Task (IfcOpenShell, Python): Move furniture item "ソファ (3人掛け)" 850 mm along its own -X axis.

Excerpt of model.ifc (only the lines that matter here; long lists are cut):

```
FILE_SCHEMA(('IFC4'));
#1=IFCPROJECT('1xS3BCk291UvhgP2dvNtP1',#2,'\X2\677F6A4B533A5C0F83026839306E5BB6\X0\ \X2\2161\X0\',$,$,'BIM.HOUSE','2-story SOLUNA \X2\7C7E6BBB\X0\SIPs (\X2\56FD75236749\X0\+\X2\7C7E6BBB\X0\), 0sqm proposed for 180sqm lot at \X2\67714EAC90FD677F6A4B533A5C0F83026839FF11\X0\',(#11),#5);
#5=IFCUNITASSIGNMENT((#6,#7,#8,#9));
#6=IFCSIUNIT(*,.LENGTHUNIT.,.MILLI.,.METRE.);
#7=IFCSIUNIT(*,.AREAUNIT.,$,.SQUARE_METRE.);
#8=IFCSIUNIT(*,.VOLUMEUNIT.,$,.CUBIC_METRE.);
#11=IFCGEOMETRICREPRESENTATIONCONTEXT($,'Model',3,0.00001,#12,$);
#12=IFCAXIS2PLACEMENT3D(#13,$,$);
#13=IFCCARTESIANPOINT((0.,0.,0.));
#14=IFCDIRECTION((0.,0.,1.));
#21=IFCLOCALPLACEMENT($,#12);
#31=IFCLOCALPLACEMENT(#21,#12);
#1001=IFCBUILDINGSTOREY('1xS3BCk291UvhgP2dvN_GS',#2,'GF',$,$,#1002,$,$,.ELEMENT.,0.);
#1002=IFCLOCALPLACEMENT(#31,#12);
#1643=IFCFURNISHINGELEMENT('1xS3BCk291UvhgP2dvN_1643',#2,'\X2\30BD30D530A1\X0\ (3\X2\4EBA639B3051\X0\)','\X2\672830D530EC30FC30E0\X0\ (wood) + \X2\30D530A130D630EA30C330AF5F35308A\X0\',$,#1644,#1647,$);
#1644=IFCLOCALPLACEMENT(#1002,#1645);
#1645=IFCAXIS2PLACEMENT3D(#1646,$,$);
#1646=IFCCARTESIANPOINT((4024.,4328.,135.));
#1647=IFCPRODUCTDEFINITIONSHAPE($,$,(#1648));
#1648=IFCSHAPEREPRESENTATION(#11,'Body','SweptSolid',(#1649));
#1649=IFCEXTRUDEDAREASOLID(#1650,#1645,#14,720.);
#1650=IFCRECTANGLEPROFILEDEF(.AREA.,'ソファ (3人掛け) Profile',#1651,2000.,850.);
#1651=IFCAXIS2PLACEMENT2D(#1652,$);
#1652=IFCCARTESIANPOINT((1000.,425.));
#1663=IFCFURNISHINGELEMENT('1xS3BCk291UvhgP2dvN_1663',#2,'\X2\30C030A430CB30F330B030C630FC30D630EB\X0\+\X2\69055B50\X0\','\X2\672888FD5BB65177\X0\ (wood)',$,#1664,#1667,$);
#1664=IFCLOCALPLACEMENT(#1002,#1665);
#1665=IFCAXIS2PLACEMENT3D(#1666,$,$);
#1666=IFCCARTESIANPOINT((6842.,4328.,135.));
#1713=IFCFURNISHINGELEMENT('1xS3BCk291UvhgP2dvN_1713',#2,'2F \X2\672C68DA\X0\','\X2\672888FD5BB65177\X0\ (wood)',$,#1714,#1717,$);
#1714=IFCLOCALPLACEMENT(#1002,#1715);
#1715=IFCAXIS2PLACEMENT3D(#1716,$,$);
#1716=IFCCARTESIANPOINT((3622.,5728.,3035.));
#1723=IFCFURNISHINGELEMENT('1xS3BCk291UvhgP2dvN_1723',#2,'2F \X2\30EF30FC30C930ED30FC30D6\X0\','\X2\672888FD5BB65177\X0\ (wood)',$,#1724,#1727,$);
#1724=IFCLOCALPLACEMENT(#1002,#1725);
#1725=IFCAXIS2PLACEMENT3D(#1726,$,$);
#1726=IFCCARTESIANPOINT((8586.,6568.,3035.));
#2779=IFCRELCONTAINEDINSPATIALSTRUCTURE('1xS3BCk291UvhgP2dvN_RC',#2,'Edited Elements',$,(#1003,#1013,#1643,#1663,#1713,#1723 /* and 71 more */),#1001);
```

```python
import ifcopenshell
import ifcopenshell.api.geometry
import ifcopenshell.util.placement
import ifcopenshell.util.unit

model = ifcopenshell.open("model.ifc")
unit_scale = ifcopenshell.util.unit.calculate_unit_scale(model)

item = model.by_guid("1xS3BCk291UvhgP2dvN_1643")
matrix = ifcopenshell.util.placement.get_local_placement(item.ObjectPlacement)
matrix[:3, 3] -= matrix[:3, 0] * 0.85 / unit_scale
ifcopenshell.api.geometry.edit_object_placement(model, product=item, matrix=matrix, is_si=False)

print(ifcopenshell.util.placement.get_local_placement(item.ObjectPlacement).round(3) + 0.0)

model.write("model_updated.ifc")
```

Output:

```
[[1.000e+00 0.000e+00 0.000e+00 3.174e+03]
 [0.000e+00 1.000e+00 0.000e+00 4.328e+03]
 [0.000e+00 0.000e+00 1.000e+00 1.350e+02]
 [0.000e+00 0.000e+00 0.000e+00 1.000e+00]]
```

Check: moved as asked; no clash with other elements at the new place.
